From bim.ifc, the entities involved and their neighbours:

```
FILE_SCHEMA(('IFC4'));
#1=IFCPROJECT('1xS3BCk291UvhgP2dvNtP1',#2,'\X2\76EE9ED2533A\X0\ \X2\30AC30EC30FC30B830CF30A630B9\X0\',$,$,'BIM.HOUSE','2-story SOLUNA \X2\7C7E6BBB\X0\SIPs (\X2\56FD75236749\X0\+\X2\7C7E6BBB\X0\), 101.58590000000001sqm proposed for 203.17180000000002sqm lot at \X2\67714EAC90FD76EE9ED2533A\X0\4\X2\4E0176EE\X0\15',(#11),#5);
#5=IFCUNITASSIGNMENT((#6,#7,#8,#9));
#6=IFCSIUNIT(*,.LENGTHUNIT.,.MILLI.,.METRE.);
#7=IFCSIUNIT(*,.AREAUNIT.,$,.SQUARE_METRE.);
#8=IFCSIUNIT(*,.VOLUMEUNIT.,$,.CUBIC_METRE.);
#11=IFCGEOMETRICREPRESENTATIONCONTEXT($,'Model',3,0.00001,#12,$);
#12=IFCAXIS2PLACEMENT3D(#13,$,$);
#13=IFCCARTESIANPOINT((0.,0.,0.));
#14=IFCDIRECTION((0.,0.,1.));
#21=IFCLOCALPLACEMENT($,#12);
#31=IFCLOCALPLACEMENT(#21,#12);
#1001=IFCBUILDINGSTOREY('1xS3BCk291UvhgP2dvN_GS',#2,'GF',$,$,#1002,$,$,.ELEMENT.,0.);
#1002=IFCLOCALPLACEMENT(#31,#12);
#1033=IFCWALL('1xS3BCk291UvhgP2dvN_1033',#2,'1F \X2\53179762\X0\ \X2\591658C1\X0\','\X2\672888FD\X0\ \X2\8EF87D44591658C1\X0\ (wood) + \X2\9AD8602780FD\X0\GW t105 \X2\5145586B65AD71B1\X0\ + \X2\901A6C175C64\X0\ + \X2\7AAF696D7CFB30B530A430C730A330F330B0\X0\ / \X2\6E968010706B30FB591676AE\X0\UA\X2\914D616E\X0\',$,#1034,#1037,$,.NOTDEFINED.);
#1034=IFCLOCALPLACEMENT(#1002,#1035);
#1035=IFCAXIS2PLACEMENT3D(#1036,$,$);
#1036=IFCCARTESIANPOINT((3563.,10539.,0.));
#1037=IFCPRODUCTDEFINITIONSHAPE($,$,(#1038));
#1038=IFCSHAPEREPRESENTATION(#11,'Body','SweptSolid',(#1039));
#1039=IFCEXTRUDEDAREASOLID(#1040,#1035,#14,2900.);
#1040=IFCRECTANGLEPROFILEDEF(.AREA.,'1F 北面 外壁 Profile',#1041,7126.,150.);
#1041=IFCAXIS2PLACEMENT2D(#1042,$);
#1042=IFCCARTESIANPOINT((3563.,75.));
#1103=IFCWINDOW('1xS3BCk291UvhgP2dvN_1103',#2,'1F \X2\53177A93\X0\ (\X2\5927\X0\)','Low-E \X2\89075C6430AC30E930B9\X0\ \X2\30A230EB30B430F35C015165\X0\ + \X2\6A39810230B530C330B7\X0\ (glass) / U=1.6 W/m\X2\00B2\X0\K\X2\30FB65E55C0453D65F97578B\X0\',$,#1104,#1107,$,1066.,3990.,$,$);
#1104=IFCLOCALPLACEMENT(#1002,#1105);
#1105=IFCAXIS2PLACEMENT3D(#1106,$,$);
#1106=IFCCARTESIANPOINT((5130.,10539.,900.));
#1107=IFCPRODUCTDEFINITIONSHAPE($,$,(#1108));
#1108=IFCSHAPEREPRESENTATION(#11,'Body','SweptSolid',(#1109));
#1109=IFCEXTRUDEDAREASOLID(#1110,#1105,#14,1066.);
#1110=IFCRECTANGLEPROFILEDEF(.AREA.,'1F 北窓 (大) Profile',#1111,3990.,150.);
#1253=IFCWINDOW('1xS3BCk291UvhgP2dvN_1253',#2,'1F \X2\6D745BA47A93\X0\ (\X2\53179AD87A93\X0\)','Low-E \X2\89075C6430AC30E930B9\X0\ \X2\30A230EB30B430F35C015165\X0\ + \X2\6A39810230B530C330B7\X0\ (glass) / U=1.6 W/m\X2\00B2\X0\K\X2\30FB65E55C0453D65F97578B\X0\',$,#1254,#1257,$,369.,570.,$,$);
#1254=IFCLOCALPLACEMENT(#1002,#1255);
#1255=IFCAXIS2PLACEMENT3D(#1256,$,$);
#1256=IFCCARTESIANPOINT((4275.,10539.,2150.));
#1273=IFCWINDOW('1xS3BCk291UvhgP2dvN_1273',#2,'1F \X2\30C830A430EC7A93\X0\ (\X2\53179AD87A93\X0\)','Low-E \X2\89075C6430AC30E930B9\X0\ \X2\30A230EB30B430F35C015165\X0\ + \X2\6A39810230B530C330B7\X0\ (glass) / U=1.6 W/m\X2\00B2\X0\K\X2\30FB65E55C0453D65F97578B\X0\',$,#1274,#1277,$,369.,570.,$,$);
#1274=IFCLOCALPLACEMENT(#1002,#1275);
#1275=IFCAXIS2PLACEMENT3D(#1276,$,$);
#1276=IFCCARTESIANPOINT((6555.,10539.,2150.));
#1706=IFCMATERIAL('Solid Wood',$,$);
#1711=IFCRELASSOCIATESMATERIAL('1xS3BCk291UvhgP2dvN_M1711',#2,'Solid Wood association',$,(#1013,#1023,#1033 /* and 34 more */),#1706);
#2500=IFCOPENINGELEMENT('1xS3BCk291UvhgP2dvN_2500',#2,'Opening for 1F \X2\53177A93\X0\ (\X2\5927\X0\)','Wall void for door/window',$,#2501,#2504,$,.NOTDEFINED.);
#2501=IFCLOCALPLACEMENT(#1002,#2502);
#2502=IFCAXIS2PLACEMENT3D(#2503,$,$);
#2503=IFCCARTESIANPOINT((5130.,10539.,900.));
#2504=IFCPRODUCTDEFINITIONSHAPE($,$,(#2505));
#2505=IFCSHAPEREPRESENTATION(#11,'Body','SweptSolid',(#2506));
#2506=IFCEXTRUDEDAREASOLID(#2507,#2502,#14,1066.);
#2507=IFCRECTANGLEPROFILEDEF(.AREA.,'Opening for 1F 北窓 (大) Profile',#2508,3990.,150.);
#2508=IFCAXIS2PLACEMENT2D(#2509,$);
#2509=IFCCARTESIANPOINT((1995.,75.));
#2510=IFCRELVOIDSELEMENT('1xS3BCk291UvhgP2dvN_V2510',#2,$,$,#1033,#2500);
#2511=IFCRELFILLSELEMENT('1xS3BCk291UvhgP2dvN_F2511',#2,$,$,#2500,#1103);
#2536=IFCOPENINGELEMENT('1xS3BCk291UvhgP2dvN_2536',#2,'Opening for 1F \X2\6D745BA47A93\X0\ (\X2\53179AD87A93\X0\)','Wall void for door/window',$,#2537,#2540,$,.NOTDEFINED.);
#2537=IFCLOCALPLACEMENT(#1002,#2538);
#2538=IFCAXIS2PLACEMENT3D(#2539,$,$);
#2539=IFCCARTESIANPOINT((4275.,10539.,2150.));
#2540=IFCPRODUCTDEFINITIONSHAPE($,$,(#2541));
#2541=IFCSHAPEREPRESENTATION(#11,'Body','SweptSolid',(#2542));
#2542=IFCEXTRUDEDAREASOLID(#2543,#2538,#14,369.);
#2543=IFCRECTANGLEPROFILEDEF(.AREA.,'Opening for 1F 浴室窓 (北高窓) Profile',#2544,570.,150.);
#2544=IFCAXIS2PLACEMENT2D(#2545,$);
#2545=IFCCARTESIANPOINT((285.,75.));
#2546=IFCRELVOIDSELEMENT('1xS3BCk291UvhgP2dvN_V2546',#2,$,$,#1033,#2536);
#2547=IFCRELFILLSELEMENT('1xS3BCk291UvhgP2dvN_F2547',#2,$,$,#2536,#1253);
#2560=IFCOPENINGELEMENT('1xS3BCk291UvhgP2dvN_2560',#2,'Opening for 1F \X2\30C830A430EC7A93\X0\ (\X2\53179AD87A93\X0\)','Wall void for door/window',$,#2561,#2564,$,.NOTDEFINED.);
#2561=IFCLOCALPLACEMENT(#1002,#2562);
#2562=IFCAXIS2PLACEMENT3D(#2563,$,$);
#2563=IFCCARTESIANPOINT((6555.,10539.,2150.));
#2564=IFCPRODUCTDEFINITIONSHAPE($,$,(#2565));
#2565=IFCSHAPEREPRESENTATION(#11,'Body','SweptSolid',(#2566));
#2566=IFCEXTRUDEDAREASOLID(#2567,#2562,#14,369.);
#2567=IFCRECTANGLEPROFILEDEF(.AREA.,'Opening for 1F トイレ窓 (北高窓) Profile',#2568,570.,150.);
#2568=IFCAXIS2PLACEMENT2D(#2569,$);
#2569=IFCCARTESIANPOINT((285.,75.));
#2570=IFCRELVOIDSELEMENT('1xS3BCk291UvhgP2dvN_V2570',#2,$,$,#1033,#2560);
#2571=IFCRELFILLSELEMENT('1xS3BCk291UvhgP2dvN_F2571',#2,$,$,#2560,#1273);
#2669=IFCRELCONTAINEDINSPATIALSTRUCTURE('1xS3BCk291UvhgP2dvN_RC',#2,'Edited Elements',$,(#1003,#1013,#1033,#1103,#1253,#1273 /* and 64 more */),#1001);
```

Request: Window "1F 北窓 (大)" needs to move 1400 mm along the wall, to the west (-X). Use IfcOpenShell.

```python
import ifcopenshell
import ifcopenshell.api.geometry
import ifcopenshell.util.placement
import ifcopenshell.util.unit

model = ifcopenshell.open("bim.ifc")
unit_scale = ifcopenshell.util.unit.calculate_unit_scale(model)

window = model.by_guid("1xS3BCk291UvhgP2dvN_1103")
opening = window.FillsVoids[0].RelatingOpeningElement
wall = opening.VoidsElements[0].RelatingBuildingElement

wall_matrix = ifcopenshell.util.placement.get_local_placement(wall.ObjectPlacement)
shift = wall_matrix[:3, 0] * -1.4 / unit_scale
before = ifcopenshell.util.placement.get_local_placement(window.ObjectPlacement)[:3, 3].copy()

# The window is not placed relative to its opening, so move both.
for product in (opening, window):
    matrix = ifcopenshell.util.placement.get_local_placement(product.ObjectPlacement)
    matrix[:3, 3] += shift
    ifcopenshell.api.geometry.edit_object_placement(model, product=product, matrix=matrix, is_si=False)

after = ifcopenshell.util.placement.get_local_placement(window.ObjectPlacement)[:3, 3]
print("window moved by", (after - before).round(3) + 0.0)

model.write("bim_rev.ifc")
```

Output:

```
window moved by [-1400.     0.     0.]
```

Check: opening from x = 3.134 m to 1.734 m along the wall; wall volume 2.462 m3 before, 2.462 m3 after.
